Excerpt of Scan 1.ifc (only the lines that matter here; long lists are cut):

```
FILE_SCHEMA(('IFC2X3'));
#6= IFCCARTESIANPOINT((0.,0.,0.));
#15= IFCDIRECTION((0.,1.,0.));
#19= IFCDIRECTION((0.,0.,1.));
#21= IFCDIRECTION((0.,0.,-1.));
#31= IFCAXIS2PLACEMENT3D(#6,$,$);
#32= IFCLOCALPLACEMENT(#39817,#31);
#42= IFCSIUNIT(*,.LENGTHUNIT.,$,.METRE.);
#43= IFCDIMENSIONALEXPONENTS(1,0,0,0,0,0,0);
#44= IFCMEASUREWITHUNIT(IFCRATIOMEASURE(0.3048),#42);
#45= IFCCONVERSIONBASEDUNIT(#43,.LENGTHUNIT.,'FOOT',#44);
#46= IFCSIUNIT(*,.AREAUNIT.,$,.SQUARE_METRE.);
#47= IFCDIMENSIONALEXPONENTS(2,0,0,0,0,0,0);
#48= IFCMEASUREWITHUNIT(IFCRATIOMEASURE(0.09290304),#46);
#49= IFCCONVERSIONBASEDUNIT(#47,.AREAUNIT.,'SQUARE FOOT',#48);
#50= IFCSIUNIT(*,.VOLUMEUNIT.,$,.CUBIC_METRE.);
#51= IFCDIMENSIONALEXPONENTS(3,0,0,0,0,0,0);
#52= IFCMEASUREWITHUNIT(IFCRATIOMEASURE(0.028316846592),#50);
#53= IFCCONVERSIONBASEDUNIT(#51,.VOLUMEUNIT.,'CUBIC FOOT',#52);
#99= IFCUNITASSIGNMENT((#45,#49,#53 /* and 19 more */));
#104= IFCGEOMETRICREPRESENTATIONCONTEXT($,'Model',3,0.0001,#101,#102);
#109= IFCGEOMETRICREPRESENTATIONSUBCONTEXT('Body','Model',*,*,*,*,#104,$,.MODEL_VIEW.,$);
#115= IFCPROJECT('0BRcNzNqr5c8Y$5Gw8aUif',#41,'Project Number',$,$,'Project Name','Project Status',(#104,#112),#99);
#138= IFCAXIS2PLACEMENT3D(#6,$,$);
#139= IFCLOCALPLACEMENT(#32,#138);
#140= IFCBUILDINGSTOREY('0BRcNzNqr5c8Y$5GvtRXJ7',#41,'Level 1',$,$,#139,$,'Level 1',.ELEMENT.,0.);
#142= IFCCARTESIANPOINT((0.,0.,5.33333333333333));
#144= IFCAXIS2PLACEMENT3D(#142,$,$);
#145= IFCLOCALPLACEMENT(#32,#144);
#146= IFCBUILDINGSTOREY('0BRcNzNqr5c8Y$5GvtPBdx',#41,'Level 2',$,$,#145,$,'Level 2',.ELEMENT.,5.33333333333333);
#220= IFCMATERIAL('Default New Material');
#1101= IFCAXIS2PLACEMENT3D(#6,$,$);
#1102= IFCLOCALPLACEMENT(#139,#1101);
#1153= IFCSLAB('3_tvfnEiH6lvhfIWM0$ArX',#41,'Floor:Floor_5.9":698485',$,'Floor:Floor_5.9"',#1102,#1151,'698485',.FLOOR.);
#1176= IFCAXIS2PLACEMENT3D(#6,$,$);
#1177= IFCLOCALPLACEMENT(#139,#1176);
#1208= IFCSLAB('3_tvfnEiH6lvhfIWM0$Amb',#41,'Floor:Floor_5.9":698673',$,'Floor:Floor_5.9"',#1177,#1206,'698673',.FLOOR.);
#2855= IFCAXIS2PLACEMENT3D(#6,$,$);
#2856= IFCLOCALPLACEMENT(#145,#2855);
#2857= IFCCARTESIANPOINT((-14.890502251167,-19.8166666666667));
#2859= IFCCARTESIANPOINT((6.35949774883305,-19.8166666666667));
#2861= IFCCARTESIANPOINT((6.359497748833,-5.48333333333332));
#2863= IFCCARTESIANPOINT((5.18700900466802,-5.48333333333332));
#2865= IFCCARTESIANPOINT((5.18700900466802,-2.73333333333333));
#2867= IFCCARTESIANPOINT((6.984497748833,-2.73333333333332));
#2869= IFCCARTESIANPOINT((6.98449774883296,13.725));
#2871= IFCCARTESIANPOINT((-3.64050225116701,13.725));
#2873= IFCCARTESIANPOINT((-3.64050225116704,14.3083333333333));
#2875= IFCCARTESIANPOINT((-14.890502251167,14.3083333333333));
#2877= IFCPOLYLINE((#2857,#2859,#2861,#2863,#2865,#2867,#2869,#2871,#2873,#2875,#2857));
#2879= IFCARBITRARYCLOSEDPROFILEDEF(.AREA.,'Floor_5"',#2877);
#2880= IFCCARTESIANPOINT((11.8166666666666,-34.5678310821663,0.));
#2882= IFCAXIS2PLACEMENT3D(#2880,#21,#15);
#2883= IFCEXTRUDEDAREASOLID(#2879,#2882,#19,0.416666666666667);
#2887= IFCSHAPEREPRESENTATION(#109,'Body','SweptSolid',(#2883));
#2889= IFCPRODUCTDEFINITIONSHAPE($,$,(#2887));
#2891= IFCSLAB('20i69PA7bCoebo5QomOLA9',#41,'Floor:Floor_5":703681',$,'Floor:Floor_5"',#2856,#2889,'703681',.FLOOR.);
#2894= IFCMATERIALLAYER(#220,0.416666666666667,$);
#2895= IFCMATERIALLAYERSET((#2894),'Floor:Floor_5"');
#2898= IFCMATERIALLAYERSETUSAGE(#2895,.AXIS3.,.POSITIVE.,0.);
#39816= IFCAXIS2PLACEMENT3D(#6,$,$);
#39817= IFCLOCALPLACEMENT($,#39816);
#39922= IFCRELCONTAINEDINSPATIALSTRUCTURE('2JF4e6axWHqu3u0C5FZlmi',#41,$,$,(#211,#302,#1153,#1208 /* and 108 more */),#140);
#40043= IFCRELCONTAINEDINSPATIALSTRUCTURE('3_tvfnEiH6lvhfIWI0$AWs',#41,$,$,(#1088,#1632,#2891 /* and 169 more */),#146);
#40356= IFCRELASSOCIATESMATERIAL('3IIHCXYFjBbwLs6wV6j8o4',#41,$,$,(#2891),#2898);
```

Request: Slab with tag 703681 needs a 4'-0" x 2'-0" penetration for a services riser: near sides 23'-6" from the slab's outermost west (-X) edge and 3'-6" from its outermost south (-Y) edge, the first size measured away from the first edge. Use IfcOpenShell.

```python
import numpy as np
import ifcopenshell
import ifcopenshell.api.feature
import ifcopenshell.api.geometry
import ifcopenshell.api.root
import ifcopenshell.geom
import ifcopenshell.util.placement
import ifcopenshell.util.representation
import ifcopenshell.util.shape
import ifcopenshell.util.unit

model = ifcopenshell.open("Scan 1.ifc")
unit_scale = ifcopenshell.util.unit.calculate_unit_scale(model)
settings = ifcopenshell.geom.settings()


def volume(element):
    """Net volume in cubic metres, openings subtracted."""
    shape = ifcopenshell.geom.create_shape(settings, element)
    return ifcopenshell.util.shape.get_volume(shape.geometry)


slab = model.by_id(2891)
before = volume(slab)

# Extent in the slab's own axes, in metres. The edges named are its -X and -Y sides.
slab_shape = ifcopenshell.geom.create_shape(settings, slab)
vertices = ifcopenshell.util.shape.get_vertices(slab_shape.geometry)
x_min, y_min, bottom = vertices.min(axis=0)
top = vertices[:, 2].max()

opening = ifcopenshell.api.root.create_entity(model, ifc_class="IfcOpeningElement", name="Services riser opening")
context = ifcopenshell.util.representation.get_context(model, "Model", "Body", "MODEL_VIEW")
width, depth = 1.2192, 0.6096
outline = [(0.0, 0.0), (width, 0.0), (width, depth), (0.0, depth), (0.0, 0.0)]
# Overshoot both faces by 50 mm so the cut is clean.
shape = ifcopenshell.api.geometry.add_slab_representation(
    model, context=context, depth=top - bottom + 0.1, polyline=outline
)
ifcopenshell.api.geometry.assign_representation(model, product=opening, representation=shape)

matrix = ifcopenshell.util.placement.get_local_placement(slab.ObjectPlacement)
matrix[:, 3] = matrix @ np.append(np.array([x_min + 7.1628, y_min + 1.0668, bottom - 0.05]) / unit_scale, 1.0)
ifcopenshell.api.geometry.edit_object_placement(model, product=opening, matrix=matrix, is_si=False)
ifcopenshell.api.feature.add_feature(model, feature=opening, element=slab)

after = volume(slab)

print(f"slab volume {before:.3f} -> {after:.3f} m3")

model.write("Scan 1_rev.ifc")
```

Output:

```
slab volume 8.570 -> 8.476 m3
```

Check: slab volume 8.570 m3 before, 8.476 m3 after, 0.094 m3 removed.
